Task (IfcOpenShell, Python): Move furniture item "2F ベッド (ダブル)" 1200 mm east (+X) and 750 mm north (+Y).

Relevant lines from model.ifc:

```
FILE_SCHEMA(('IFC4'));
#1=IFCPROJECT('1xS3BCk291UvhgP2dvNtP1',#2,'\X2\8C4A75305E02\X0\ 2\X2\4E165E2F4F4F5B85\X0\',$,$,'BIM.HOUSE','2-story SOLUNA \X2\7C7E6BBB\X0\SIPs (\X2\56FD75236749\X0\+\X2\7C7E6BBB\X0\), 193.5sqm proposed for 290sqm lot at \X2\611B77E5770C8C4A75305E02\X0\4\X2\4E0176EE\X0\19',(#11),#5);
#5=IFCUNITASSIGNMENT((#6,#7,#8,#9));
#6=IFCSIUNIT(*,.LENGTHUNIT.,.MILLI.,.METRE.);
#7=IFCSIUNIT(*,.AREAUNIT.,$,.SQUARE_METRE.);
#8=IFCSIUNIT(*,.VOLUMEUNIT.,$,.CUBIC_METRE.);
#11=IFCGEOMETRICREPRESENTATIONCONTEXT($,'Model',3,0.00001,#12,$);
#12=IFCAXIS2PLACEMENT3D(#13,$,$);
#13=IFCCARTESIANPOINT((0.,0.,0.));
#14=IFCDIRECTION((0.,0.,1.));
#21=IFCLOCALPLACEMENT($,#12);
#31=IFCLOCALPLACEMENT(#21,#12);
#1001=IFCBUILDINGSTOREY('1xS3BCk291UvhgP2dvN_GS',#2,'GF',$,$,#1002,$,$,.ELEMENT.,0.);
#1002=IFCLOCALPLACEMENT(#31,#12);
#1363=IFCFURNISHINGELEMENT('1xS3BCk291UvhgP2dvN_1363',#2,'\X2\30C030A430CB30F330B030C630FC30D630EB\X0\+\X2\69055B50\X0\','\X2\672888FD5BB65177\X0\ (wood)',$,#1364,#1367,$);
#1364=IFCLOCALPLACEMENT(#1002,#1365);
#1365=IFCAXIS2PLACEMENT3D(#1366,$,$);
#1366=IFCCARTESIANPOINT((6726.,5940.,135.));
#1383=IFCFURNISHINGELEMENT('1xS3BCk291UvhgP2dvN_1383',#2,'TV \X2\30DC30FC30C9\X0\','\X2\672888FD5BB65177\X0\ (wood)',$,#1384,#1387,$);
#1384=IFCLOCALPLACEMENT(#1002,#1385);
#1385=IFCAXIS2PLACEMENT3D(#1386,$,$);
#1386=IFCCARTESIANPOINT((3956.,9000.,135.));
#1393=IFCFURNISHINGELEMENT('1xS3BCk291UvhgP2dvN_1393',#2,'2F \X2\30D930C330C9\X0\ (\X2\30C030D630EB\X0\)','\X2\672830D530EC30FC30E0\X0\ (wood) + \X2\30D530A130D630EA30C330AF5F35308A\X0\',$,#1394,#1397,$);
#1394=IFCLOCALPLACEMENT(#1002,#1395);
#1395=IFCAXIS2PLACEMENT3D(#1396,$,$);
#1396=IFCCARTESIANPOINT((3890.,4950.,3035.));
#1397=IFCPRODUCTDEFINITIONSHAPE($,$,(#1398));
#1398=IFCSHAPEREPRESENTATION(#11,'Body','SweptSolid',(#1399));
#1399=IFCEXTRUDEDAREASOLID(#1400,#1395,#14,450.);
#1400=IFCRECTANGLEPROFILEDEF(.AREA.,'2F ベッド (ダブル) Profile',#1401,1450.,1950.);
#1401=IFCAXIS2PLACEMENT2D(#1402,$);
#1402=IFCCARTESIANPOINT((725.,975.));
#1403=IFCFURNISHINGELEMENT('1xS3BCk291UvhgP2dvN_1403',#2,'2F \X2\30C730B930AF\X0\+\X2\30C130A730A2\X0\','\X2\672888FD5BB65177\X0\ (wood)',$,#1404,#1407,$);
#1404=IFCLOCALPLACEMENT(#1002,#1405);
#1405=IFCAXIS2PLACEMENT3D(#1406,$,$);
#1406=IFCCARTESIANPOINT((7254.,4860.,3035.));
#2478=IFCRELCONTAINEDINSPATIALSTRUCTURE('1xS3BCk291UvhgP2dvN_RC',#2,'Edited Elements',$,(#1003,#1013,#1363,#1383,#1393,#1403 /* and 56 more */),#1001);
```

```python
import ifcopenshell
import ifcopenshell.api.geometry
import ifcopenshell.util.placement
import ifcopenshell.util.unit

model = ifcopenshell.open("model.ifc")
unit_scale = ifcopenshell.util.unit.calculate_unit_scale(model)

item = model.by_id(1393)
matrix = ifcopenshell.util.placement.get_local_placement(item.ObjectPlacement)
matrix[0, 3] += 1.2 / unit_scale
matrix[1, 3] += 0.75 / unit_scale
ifcopenshell.api.geometry.edit_object_placement(model, product=item, matrix=matrix, is_si=False)

print(ifcopenshell.util.placement.get_local_placement(item.ObjectPlacement).round(3) + 0.0)

model.write("model_v2.ifc")
```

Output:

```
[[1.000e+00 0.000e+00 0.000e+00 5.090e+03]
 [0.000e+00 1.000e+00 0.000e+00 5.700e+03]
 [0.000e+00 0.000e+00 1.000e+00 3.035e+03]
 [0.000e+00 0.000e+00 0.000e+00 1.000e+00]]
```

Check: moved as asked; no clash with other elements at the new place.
